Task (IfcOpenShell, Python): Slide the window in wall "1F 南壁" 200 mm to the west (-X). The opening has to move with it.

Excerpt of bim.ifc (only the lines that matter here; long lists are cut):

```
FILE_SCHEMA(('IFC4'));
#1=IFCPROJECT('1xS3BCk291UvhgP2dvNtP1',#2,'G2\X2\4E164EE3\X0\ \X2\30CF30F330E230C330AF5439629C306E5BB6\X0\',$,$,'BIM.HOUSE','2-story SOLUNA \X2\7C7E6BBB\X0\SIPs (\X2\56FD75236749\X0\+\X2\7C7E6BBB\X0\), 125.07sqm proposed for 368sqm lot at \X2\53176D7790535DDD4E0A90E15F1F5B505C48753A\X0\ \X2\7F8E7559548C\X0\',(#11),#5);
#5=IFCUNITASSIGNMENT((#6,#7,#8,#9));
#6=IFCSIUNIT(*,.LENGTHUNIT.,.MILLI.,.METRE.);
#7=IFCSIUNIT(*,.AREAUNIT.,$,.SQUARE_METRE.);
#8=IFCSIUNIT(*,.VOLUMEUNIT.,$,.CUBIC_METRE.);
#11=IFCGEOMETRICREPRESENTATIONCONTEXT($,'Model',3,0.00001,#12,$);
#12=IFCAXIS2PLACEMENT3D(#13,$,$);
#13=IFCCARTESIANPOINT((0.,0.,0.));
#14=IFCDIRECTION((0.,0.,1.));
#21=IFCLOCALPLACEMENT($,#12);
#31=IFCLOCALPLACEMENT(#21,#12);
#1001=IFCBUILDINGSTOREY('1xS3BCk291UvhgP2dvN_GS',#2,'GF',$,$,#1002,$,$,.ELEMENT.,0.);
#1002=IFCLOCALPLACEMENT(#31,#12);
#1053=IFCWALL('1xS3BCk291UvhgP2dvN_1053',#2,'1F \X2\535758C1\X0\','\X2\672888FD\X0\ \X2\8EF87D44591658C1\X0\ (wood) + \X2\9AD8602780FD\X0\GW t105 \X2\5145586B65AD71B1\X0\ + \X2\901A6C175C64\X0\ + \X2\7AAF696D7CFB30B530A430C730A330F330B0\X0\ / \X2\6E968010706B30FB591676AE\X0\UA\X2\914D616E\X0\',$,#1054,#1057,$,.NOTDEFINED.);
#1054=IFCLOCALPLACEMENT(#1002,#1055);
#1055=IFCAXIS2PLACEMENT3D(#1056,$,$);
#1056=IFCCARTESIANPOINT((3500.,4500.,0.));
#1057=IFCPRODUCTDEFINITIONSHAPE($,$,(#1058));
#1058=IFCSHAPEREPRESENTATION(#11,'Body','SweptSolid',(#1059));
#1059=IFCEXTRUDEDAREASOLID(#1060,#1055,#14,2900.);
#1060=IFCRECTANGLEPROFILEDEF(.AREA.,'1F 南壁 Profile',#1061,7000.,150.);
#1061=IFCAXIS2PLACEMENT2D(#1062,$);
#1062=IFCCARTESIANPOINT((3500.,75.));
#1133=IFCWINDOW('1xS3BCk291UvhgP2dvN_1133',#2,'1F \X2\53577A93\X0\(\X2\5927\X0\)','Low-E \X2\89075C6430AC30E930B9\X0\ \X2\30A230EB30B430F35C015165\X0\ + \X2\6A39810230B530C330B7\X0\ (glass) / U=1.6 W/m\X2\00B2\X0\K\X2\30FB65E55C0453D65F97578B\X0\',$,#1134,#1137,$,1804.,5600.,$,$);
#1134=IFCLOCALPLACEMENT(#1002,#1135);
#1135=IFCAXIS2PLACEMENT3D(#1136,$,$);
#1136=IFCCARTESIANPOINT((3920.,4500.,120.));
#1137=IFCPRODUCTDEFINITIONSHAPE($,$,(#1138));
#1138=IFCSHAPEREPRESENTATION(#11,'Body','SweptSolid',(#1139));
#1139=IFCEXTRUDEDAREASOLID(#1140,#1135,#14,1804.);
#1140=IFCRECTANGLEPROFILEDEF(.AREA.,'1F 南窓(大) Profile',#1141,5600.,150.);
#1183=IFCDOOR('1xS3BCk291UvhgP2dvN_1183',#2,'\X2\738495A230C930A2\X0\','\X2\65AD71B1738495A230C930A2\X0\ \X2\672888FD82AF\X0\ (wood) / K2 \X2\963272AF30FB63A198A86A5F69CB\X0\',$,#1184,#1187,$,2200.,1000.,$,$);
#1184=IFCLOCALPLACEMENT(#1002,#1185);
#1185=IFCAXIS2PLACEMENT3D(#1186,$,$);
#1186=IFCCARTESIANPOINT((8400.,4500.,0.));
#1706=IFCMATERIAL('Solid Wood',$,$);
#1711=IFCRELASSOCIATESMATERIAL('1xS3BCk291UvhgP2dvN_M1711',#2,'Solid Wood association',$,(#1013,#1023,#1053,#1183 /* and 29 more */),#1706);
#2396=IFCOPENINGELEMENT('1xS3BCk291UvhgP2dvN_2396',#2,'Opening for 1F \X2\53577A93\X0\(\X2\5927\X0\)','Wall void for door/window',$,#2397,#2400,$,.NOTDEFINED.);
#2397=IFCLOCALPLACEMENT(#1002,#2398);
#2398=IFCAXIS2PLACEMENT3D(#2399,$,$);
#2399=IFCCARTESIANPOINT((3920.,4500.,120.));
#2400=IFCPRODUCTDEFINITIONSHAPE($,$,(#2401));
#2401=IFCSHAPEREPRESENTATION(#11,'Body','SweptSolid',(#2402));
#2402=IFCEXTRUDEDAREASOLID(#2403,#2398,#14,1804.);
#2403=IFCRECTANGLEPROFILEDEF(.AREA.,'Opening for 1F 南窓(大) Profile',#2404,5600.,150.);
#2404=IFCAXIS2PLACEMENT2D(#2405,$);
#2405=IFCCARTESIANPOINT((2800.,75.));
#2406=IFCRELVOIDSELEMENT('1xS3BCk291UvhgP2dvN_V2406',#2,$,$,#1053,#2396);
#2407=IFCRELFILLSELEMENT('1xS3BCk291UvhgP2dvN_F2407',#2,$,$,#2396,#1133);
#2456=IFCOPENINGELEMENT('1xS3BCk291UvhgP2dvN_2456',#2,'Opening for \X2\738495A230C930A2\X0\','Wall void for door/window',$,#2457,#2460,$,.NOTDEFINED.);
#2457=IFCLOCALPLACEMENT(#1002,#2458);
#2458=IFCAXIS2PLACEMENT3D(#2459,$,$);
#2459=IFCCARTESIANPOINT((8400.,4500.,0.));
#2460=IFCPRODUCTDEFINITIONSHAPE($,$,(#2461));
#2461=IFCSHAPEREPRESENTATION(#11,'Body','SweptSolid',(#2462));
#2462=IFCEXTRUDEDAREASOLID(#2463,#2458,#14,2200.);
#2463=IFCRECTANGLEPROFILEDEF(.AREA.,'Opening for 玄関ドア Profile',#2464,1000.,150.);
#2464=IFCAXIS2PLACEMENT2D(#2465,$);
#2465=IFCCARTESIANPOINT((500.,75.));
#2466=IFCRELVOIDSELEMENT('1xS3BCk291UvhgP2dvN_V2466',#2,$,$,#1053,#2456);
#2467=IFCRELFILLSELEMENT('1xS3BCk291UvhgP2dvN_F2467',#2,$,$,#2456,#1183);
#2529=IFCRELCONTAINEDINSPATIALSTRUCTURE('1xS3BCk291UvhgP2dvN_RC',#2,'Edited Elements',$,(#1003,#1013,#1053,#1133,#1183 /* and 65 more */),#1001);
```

```python
import ifcopenshell
import ifcopenshell.api.geometry
import ifcopenshell.util.placement

model = ifcopenshell.open("bim.ifc")

window = model.by_id(1133)
opening = window.FillsVoids[0].RelatingOpeningElement
wall = opening.VoidsElements[0].RelatingBuildingElement

wall_matrix = ifcopenshell.util.placement.get_local_placement(wall.ObjectPlacement)
shift = wall_matrix[:3, 0] * -200.0
before = ifcopenshell.util.placement.get_local_placement(window.ObjectPlacement)[:3, 3].copy()

# The window is not placed relative to its opening, so move both.
for product in (opening, window):
    matrix = ifcopenshell.util.placement.get_local_placement(product.ObjectPlacement)
    matrix[:3, 3] += shift
    ifcopenshell.api.geometry.edit_object_placement(model, product=product, matrix=matrix, is_si=False)

after = ifcopenshell.util.placement.get_local_placement(window.ObjectPlacement)[:3, 3]
print("window moved by", (after - before).round(3) + 0.0)

model.write("bim_edited.ifc")
```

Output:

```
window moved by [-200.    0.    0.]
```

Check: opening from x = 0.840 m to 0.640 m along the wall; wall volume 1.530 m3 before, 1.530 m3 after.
